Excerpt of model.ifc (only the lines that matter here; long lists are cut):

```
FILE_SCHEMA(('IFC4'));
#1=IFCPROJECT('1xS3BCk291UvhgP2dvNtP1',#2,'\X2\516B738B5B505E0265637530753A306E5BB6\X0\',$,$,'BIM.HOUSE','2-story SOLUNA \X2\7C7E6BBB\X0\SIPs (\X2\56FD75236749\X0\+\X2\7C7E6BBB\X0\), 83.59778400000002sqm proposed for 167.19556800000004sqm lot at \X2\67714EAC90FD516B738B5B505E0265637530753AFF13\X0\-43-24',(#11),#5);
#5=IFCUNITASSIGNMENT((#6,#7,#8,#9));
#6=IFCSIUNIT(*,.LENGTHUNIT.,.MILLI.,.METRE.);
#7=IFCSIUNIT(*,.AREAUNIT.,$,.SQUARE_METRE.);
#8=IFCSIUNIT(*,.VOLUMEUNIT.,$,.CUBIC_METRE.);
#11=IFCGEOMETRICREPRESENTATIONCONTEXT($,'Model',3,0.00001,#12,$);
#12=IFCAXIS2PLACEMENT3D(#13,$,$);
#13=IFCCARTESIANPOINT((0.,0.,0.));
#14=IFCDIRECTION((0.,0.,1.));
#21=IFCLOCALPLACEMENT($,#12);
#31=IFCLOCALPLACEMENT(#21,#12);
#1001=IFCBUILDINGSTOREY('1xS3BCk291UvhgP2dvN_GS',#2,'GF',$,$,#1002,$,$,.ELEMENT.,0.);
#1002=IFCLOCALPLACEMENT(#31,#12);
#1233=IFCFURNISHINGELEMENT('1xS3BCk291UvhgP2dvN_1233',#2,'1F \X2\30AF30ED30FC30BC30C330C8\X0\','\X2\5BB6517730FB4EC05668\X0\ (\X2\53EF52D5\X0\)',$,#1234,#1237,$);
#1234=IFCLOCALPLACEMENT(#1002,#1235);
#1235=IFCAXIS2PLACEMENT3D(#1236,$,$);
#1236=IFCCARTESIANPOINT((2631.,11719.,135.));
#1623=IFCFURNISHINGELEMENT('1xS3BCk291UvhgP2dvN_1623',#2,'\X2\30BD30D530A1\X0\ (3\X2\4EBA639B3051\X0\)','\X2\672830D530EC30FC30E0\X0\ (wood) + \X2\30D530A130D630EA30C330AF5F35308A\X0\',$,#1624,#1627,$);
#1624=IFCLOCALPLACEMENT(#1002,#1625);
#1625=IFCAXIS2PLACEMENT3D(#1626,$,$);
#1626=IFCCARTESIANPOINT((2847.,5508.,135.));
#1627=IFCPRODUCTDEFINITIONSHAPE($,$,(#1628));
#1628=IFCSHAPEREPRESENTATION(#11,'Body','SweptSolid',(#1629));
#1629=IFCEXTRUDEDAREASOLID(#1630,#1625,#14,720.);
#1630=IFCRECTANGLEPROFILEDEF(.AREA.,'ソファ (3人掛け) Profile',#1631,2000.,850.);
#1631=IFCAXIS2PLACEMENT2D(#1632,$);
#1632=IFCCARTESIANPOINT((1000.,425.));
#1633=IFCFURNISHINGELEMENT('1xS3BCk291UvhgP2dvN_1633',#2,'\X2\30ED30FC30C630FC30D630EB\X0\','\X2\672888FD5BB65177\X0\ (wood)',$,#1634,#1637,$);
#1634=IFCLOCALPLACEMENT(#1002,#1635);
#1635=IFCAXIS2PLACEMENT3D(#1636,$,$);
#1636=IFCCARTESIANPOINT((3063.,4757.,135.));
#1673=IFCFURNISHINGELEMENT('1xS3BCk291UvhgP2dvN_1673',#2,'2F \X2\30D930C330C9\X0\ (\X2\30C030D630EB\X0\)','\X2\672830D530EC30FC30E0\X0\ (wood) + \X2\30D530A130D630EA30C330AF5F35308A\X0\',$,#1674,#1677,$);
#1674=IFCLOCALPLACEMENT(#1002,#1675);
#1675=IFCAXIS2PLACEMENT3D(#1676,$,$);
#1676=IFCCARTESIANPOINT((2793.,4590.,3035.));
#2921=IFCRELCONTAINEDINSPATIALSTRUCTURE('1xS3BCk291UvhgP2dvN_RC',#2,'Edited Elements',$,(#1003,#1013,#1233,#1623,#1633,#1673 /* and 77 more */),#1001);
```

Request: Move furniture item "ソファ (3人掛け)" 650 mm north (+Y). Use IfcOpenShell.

```python
import ifcopenshell
import ifcopenshell.api.geometry
import ifcopenshell.util.placement
import ifcopenshell.util.unit

model = ifcopenshell.open("model.ifc")
unit_scale = ifcopenshell.util.unit.calculate_unit_scale(model)

item = model.by_guid("1xS3BCk291UvhgP2dvN_1623")
matrix = ifcopenshell.util.placement.get_local_placement(item.ObjectPlacement)
matrix[1, 3] += 0.65 / unit_scale
ifcopenshell.api.geometry.edit_object_placement(model, product=item, matrix=matrix, is_si=False)

print(ifcopenshell.util.placement.get_local_placement(item.ObjectPlacement).round(3) + 0.0)

model.write("model-out.ifc")
```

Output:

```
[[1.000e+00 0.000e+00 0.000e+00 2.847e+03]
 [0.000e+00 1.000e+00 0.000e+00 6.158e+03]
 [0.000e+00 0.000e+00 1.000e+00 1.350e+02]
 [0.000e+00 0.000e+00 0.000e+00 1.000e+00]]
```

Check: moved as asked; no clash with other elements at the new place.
